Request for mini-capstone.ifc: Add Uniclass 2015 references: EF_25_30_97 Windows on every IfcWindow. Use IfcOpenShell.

First a look at what the model holds.

```python
import ifcopenshell

model = ifcopenshell.open("mini-capstone.ifc")
print(model.schema)
print("classifications:", [c.Name for c in model.by_type("IfcClassification")])
for ifc_class in ("IfcDoor", "IfcRoof", "IfcStair", "IfcWall", "IfcWindow"):
    print(ifc_class, len(model.by_type(ifc_class)))
```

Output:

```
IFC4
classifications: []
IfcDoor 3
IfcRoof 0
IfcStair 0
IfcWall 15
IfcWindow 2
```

```python
import ifcopenshell
import ifcopenshell.api.classification

model = ifcopenshell.open("mini-capstone.ifc")

system = ifcopenshell.api.classification.add_classification(model, classification="Uniclass 2015")

codes = {
    "IfcWindow": ("EF_25_30_97", "Windows"),
}
for ifc_class, (code, name) in codes.items():
    products = model.by_type(ifc_class)
    ifcopenshell.api.classification.add_reference(
        model, products=products, classification=system, identification=code, name=name
    )
    print(code, len(products))

model.write("mini-capstone_edited.ifc")
```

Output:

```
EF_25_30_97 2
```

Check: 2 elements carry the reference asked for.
